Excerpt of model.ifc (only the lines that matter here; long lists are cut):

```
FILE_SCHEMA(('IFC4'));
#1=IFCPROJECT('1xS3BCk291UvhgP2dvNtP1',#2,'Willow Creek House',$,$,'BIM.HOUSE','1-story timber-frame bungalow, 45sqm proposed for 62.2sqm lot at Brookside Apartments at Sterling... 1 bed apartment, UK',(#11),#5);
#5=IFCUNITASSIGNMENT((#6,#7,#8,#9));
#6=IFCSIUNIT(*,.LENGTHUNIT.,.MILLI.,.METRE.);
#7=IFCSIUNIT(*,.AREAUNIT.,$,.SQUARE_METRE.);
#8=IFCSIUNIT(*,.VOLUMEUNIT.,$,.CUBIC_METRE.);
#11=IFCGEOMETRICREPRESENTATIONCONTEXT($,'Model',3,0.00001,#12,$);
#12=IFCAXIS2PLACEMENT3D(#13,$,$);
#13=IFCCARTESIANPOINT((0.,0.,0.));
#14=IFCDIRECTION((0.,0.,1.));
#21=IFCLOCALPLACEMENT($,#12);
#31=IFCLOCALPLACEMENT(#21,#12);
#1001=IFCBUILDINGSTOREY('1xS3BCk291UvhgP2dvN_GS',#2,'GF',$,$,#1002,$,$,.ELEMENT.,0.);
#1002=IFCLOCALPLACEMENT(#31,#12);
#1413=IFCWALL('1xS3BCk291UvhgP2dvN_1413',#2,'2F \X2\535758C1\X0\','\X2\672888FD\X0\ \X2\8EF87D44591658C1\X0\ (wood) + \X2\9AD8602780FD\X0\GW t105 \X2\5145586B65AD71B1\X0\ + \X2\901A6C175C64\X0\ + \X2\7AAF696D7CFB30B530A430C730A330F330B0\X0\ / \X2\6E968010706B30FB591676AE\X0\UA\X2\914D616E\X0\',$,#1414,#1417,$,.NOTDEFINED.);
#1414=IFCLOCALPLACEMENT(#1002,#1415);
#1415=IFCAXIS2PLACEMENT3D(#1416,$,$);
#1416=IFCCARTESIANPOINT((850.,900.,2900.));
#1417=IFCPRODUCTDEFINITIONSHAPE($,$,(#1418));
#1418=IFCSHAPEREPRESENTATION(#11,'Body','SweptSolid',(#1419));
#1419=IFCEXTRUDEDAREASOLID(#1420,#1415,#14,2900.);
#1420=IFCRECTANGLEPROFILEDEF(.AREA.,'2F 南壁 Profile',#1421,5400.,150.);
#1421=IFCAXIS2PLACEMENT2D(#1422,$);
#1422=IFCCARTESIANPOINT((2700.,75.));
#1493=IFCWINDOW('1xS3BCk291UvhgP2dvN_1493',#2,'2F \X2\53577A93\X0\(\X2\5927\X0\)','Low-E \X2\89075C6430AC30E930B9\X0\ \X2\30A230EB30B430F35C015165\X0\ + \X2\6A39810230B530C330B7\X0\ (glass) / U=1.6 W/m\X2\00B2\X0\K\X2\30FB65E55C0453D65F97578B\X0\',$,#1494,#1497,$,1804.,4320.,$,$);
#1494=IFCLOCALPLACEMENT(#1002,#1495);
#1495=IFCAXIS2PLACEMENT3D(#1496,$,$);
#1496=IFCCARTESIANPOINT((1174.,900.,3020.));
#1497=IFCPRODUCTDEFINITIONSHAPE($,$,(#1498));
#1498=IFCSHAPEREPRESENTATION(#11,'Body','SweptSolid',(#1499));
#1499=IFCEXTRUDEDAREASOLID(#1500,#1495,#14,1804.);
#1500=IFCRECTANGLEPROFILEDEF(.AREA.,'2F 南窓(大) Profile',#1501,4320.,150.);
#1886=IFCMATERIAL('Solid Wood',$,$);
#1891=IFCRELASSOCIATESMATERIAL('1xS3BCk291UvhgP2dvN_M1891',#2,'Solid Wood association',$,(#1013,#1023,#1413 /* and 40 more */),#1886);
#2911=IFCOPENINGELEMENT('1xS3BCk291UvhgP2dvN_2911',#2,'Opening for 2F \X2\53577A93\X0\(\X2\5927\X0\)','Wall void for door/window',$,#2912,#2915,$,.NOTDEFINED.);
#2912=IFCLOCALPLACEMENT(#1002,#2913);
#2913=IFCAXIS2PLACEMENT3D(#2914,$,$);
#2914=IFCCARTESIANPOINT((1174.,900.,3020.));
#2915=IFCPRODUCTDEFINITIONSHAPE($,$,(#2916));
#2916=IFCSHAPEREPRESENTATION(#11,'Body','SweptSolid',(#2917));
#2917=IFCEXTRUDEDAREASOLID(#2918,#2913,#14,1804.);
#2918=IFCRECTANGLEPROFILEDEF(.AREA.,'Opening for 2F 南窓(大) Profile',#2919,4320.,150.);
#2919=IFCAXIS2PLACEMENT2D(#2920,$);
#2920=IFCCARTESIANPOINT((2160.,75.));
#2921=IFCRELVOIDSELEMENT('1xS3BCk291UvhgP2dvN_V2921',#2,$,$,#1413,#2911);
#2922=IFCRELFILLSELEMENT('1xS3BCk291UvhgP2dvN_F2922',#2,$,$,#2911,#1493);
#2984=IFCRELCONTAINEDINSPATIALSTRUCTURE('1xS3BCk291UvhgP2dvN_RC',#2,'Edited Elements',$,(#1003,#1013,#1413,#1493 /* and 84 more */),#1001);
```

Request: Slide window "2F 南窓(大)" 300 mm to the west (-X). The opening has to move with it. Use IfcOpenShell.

```python
import ifcopenshell
import ifcopenshell.api.geometry
import ifcopenshell.util.placement

model = ifcopenshell.open("model.ifc")

window = model.by_guid("1xS3BCk291UvhgP2dvN_1493")
opening = window.FillsVoids[0].RelatingOpeningElement
wall = opening.VoidsElements[0].RelatingBuildingElement

wall_matrix = ifcopenshell.util.placement.get_local_placement(wall.ObjectPlacement)
shift = wall_matrix[:3, 0] * -300.0
before = ifcopenshell.util.placement.get_local_placement(window.ObjectPlacement)[:3, 3].copy()

# The window is not placed relative to its opening, so move both.
for product in (opening, window):
    matrix = ifcopenshell.util.placement.get_local_placement(product.ObjectPlacement)
    matrix[:3, 3] += shift
    ifcopenshell.api.geometry.edit_object_placement(model, product=product, matrix=matrix, is_si=False)

after = ifcopenshell.util.placement.get_local_placement(window.ObjectPlacement)[:3, 3]
print("window moved by", (after - before).round(3) + 0.0)

model.write("model_edited.ifc")
```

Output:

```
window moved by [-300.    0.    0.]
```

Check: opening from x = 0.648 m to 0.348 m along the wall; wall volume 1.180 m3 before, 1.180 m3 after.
